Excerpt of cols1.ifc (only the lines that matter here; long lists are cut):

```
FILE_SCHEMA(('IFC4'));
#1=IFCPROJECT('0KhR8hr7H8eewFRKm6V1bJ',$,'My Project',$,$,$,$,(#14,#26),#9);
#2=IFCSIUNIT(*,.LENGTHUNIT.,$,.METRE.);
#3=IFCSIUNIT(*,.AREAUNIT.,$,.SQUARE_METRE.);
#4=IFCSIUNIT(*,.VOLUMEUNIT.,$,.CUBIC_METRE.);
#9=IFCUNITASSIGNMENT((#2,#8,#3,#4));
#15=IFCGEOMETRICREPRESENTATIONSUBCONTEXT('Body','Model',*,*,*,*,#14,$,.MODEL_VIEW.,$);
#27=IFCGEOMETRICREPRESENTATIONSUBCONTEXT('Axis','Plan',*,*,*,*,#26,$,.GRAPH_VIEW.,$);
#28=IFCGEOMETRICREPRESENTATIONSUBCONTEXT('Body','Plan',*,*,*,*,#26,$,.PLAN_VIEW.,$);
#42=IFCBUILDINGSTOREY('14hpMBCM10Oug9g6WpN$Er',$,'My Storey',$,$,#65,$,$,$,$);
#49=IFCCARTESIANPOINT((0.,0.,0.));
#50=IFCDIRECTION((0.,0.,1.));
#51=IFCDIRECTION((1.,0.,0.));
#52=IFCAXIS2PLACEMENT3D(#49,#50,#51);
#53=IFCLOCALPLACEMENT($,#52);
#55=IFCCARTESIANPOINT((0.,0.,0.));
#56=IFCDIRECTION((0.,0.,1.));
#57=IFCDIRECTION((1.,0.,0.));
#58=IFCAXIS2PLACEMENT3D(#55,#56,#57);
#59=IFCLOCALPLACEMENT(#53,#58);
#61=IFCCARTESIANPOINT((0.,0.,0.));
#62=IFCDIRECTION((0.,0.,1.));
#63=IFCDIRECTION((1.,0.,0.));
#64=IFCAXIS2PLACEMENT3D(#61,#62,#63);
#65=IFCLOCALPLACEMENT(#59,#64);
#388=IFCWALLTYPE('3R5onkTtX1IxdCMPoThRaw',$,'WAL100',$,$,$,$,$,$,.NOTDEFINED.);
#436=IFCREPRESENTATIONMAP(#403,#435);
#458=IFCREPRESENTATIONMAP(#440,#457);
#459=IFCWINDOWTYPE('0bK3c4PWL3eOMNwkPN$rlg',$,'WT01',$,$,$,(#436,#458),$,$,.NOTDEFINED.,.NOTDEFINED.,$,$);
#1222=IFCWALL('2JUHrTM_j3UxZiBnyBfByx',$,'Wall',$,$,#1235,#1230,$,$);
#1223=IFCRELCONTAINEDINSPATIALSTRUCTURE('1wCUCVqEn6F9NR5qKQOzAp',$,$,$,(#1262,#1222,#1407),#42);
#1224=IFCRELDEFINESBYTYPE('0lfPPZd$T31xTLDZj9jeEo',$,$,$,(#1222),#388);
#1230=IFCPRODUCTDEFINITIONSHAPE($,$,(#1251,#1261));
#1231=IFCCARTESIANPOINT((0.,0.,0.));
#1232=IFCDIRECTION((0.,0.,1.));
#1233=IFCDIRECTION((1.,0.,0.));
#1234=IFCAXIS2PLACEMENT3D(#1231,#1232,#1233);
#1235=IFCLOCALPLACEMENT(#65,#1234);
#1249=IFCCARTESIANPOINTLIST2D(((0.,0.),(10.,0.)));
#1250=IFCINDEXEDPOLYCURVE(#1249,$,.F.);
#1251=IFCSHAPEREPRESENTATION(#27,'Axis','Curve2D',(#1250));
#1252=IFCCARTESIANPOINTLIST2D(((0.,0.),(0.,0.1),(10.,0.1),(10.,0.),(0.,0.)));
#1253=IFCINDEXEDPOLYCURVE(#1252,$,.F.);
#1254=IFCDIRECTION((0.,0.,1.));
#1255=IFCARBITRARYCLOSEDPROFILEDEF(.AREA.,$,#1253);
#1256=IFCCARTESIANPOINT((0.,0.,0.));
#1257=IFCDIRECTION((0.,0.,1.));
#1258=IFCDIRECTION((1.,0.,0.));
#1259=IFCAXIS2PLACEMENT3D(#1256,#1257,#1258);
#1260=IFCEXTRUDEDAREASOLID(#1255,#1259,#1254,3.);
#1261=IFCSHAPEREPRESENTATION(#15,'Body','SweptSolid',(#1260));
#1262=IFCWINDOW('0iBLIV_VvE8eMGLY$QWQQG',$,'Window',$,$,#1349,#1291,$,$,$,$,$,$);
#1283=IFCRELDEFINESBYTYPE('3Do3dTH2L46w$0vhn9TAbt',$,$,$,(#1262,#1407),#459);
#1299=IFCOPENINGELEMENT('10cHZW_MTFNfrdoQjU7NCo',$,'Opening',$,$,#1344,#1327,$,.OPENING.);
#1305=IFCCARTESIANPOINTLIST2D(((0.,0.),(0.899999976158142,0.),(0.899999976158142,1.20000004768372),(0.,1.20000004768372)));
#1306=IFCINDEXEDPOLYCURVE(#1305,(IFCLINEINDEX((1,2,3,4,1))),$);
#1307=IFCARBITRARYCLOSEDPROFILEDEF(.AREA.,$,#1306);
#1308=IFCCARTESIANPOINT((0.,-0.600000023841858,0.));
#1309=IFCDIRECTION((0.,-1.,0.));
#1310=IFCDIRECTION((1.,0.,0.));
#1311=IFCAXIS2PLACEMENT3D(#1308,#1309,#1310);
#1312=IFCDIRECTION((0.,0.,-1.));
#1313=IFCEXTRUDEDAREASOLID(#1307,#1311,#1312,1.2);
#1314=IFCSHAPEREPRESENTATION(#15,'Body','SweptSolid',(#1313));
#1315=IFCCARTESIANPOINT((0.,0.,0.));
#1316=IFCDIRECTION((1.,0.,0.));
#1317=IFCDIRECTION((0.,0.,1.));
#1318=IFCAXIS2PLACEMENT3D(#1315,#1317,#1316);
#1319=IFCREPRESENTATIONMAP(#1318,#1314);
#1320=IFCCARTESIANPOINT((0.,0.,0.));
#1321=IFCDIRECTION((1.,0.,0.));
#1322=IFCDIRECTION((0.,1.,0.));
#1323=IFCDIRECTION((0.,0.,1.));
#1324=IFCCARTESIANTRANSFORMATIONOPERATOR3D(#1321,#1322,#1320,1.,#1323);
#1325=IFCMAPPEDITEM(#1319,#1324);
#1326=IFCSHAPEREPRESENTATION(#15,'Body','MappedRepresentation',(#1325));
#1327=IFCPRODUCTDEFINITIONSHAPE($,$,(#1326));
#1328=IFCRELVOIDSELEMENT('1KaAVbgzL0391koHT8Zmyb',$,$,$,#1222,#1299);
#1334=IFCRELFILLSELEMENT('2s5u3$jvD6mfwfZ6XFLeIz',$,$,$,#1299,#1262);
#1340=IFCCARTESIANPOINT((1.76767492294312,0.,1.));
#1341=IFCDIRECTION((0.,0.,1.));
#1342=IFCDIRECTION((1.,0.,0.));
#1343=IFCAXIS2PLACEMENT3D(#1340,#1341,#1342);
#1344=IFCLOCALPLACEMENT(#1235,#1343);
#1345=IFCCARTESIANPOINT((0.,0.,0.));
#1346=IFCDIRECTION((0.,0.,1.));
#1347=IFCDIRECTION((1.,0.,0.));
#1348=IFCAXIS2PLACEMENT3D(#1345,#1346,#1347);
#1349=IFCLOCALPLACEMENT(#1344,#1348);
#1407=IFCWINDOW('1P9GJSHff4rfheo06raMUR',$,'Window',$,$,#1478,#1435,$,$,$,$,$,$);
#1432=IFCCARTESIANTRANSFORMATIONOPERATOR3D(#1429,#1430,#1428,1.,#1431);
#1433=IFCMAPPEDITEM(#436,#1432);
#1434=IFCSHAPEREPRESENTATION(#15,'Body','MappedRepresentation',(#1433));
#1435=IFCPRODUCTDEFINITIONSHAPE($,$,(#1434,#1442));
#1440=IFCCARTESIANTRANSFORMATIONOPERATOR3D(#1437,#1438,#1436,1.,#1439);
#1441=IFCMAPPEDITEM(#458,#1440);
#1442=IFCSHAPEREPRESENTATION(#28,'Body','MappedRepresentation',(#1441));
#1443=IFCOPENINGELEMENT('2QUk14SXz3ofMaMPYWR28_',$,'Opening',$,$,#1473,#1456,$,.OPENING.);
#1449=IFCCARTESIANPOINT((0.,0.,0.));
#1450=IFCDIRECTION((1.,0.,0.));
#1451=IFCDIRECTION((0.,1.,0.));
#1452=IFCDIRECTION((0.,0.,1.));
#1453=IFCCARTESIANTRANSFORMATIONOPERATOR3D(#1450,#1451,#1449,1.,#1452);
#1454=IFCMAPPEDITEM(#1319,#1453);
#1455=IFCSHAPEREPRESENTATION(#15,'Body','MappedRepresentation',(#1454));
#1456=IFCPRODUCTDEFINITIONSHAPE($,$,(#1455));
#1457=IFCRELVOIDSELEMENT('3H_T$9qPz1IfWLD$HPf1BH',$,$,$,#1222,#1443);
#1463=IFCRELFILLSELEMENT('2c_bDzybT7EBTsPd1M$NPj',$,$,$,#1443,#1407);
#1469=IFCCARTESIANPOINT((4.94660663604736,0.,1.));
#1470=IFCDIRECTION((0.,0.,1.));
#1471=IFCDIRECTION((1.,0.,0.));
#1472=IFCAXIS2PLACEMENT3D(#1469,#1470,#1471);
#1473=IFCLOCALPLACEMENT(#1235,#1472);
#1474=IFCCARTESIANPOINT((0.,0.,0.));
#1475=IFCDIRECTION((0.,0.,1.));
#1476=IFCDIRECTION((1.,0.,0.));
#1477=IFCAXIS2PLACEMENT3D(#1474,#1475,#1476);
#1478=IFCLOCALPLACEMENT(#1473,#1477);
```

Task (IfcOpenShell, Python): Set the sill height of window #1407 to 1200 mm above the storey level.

```python
import numpy as np
import ifcopenshell
import ifcopenshell.api.geometry
import ifcopenshell.geom
import ifcopenshell.util.element
import ifcopenshell.util.placement
import ifcopenshell.util.shape
import ifcopenshell.util.unit

model = ifcopenshell.open("cols1.ifc")
unit_scale = ifcopenshell.util.unit.calculate_unit_scale(model)

window = model.by_guid("1P9GJSHff4rfheo06raMUR")
opening = window.FillsVoids[0].RelatingOpeningElement
storey = ifcopenshell.util.element.get_container(window, ifc_class="IfcBuildingStorey")
level = ifcopenshell.util.placement.get_local_placement(storey.ObjectPlacement)[2, 3]

# The opening's origin need not be at the sill, so measure its lowest point.
shape = ifcopenshell.geom.create_shape(ifcopenshell.geom.settings(), opening)
bottom = ifcopenshell.util.shape.get_shape_bottom_elevation(shape, shape.geometry) / unit_scale
dz = level + 1.2 / unit_scale - bottom

shift = np.array([0.0, 0.0, dz])
# The window is placed relative to its opening, so it follows when the opening moves.
matrix = ifcopenshell.util.placement.get_local_placement(opening.ObjectPlacement)
matrix[:3, 3] += shift
ifcopenshell.api.geometry.edit_object_placement(
    model, product=opening, matrix=matrix, is_si=False, should_transform_children=True
)

print(f"moved by {dz * unit_scale:+.3f} m")

model.write("cols1_edited.ifc")
```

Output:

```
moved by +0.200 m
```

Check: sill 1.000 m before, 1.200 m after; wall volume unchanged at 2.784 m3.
